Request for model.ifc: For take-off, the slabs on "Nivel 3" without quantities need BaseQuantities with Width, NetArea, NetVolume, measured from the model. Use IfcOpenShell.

First a look at what the model holds.

```python
import ifcopenshell
import ifcopenshell.util.element
import ifcopenshell.util.unit

model = ifcopenshell.open("model.ifc")
print(model.schema)
for unit_type in ("LENGTHUNIT", "AREAUNIT", "VOLUMEUNIT"):
    print(unit_type, ifcopenshell.util.unit.calculate_unit_scale(model, unit_type))
storey = next(s for s in model.by_type("IfcBuildingStorey") if s.Name == "Nivel 3")
slabs = [e for e in ifcopenshell.util.element.get_decomposition(storey) if e.is_a("IfcSlab")]
for e in sorted(slabs, key=lambda e: e.id()):
    print(e.id(), e.is_a(), e.Name, list(ifcopenshell.util.element.get_psets(e, qtos_only=True)), sep=" | ")
```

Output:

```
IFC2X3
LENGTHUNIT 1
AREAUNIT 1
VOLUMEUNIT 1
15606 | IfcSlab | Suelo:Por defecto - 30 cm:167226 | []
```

```python
import ifcopenshell
import ifcopenshell.api.pset
import ifcopenshell.geom
import ifcopenshell.util.element
import ifcopenshell.util.shape
import ifcopenshell.util.unit

model = ifcopenshell.open("model.ifc")
unit_scale = ifcopenshell.util.unit.calculate_unit_scale(model)
area_scale = ifcopenshell.util.unit.calculate_unit_scale(model, "AREAUNIT")
volume_scale = ifcopenshell.util.unit.calculate_unit_scale(model, "VOLUMEUNIT")
settings = ifcopenshell.geom.settings()

storey = next(s for s in model.by_type("IfcBuildingStorey") if s.Name == "Nivel 3")
slabs = [e for e in ifcopenshell.util.element.get_decomposition(storey) if e.is_a("IfcSlab")]

for e in sorted(slabs, key=lambda e: e.id()):
    if ifcopenshell.util.element.get_psets(e, qtos_only=True, should_inherit=False):
        continue
    # Geometry comes back in metres, in the element's own axes.
    shape = ifcopenshell.geom.create_shape(settings, e)
    values = {
        "Width": ifcopenshell.util.shape.get_z(shape.geometry) / unit_scale,
        "NetArea": ifcopenshell.util.shape.get_footprint_area(shape.geometry) / area_scale,
        "NetVolume": ifcopenshell.util.shape.get_volume(shape.geometry) / volume_scale,
    }
    qto = ifcopenshell.api.pset.add_qto(model, product=e, name="BaseQuantities")
    ifcopenshell.api.pset.edit_qto(model, qto=qto, properties=values)
    print(e.id(), {k: round(v, 3) for k, v in values.items()})

model.write("model-out.ifc")
```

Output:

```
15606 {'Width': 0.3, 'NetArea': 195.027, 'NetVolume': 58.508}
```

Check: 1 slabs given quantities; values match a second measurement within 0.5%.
